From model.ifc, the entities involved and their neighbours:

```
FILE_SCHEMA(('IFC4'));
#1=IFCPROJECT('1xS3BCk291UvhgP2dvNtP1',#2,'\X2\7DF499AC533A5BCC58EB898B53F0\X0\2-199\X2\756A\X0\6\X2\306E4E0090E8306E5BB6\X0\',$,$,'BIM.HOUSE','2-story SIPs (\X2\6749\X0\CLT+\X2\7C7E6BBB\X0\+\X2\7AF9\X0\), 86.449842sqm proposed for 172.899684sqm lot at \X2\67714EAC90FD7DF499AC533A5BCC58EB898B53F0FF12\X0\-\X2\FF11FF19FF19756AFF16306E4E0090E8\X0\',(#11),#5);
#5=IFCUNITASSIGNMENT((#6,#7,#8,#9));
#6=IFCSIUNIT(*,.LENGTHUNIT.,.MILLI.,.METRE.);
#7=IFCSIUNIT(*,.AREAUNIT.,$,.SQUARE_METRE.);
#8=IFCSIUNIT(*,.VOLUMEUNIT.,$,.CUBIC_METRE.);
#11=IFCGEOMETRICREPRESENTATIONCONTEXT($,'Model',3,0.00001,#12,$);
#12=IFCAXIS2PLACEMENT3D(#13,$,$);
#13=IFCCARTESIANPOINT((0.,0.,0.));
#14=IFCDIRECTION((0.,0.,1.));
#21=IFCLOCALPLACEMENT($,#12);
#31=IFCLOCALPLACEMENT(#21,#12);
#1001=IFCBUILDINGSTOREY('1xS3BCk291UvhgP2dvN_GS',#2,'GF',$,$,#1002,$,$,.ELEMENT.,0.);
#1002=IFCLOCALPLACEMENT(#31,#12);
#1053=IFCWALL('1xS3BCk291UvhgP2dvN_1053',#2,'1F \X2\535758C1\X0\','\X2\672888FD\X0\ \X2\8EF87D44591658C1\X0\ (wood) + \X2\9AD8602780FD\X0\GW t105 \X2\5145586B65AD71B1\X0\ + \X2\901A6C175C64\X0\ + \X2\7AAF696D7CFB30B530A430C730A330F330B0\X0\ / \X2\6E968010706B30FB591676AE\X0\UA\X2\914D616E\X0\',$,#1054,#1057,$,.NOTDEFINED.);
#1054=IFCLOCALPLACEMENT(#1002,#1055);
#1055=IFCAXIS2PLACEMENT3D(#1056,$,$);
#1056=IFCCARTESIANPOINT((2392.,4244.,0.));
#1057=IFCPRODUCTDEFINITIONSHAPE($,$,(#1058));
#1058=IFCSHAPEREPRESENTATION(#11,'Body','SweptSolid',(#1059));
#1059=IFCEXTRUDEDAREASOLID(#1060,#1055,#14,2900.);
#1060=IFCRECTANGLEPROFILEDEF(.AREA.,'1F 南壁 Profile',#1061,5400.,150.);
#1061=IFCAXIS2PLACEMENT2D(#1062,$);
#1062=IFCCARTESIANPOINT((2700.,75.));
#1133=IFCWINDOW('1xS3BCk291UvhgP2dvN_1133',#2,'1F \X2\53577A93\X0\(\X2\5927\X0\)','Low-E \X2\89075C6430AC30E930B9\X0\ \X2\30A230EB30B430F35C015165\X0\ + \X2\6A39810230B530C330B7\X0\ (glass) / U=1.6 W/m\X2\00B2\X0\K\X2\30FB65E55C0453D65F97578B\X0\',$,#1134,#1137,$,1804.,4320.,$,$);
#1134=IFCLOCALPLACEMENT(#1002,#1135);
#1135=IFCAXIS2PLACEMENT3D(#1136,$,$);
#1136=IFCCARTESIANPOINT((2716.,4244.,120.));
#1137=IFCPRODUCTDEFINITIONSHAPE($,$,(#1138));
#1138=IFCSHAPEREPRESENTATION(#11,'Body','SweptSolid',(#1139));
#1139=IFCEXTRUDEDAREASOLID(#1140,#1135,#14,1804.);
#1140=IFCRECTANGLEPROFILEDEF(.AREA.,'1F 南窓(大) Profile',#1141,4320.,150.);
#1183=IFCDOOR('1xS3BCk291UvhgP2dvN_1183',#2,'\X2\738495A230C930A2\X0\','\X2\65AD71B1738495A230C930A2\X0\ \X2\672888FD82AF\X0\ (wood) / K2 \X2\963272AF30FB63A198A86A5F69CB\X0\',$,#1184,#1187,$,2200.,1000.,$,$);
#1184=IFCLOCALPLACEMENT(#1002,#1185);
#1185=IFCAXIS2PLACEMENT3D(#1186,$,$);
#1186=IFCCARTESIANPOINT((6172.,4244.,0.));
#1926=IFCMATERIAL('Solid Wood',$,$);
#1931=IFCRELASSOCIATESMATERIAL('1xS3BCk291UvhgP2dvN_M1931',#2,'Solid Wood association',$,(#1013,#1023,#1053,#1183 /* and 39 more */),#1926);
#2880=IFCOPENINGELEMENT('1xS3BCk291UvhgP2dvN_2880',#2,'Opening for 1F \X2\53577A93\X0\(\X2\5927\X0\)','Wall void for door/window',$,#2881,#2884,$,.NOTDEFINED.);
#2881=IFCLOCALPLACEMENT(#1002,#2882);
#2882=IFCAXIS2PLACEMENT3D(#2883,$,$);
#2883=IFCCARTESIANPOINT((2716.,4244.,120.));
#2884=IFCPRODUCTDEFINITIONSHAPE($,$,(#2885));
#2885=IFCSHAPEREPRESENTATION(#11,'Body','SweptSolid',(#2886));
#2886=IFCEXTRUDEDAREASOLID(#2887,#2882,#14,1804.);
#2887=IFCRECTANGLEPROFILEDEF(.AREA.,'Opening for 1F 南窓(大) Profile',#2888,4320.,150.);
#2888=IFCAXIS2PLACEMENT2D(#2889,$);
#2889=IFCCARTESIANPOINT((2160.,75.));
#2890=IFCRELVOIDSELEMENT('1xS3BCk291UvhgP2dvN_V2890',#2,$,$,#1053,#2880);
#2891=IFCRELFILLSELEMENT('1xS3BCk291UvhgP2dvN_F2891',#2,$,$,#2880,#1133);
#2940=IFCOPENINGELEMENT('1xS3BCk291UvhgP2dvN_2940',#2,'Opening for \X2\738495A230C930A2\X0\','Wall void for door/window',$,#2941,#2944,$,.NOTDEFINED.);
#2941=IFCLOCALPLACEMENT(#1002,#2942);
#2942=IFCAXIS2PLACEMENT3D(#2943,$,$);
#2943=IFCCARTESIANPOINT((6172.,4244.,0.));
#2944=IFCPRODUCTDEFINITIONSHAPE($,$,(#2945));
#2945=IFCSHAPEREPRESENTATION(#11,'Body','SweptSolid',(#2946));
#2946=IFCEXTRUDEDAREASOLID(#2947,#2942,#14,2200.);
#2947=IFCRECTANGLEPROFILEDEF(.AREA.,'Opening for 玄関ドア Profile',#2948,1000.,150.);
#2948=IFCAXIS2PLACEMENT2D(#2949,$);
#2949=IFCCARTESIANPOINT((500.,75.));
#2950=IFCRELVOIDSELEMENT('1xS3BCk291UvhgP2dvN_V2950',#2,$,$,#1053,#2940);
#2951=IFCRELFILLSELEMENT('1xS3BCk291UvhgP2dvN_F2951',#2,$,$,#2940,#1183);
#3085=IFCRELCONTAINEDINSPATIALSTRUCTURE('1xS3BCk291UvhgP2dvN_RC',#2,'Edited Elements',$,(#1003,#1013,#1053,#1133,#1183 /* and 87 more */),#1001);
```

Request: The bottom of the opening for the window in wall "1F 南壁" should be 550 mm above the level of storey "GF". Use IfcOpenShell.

```python
import numpy as np
import ifcopenshell
import ifcopenshell.api.geometry
import ifcopenshell.geom
import ifcopenshell.util.element
import ifcopenshell.util.placement
import ifcopenshell.util.shape
import ifcopenshell.util.unit

model = ifcopenshell.open("model.ifc")
unit_scale = ifcopenshell.util.unit.calculate_unit_scale(model)

window = model.by_guid("1xS3BCk291UvhgP2dvN_1133")
opening = window.FillsVoids[0].RelatingOpeningElement
storey = ifcopenshell.util.element.get_container(window, ifc_class="IfcBuildingStorey")
level = ifcopenshell.util.placement.get_local_placement(storey.ObjectPlacement)[2, 3]

# The opening's origin need not be at the sill, so measure its lowest point.
shape = ifcopenshell.geom.create_shape(ifcopenshell.geom.settings(), opening)
bottom = ifcopenshell.util.shape.get_shape_bottom_elevation(shape, shape.geometry) / unit_scale
dz = level + 0.55 / unit_scale - bottom

shift = np.array([0.0, 0.0, dz])
# The window is not placed relative to its opening, so move both.
for product in (opening, window):
    matrix = ifcopenshell.util.placement.get_local_placement(product.ObjectPlacement)
    matrix[:3, 3] += shift
    ifcopenshell.api.geometry.edit_object_placement(model, product=product, matrix=matrix, is_si=False)

print(f"moved by {dz * unit_scale:+.3f} m")

model.write("model_updated.ifc")
```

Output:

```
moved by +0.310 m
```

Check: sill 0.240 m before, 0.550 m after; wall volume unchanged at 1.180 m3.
